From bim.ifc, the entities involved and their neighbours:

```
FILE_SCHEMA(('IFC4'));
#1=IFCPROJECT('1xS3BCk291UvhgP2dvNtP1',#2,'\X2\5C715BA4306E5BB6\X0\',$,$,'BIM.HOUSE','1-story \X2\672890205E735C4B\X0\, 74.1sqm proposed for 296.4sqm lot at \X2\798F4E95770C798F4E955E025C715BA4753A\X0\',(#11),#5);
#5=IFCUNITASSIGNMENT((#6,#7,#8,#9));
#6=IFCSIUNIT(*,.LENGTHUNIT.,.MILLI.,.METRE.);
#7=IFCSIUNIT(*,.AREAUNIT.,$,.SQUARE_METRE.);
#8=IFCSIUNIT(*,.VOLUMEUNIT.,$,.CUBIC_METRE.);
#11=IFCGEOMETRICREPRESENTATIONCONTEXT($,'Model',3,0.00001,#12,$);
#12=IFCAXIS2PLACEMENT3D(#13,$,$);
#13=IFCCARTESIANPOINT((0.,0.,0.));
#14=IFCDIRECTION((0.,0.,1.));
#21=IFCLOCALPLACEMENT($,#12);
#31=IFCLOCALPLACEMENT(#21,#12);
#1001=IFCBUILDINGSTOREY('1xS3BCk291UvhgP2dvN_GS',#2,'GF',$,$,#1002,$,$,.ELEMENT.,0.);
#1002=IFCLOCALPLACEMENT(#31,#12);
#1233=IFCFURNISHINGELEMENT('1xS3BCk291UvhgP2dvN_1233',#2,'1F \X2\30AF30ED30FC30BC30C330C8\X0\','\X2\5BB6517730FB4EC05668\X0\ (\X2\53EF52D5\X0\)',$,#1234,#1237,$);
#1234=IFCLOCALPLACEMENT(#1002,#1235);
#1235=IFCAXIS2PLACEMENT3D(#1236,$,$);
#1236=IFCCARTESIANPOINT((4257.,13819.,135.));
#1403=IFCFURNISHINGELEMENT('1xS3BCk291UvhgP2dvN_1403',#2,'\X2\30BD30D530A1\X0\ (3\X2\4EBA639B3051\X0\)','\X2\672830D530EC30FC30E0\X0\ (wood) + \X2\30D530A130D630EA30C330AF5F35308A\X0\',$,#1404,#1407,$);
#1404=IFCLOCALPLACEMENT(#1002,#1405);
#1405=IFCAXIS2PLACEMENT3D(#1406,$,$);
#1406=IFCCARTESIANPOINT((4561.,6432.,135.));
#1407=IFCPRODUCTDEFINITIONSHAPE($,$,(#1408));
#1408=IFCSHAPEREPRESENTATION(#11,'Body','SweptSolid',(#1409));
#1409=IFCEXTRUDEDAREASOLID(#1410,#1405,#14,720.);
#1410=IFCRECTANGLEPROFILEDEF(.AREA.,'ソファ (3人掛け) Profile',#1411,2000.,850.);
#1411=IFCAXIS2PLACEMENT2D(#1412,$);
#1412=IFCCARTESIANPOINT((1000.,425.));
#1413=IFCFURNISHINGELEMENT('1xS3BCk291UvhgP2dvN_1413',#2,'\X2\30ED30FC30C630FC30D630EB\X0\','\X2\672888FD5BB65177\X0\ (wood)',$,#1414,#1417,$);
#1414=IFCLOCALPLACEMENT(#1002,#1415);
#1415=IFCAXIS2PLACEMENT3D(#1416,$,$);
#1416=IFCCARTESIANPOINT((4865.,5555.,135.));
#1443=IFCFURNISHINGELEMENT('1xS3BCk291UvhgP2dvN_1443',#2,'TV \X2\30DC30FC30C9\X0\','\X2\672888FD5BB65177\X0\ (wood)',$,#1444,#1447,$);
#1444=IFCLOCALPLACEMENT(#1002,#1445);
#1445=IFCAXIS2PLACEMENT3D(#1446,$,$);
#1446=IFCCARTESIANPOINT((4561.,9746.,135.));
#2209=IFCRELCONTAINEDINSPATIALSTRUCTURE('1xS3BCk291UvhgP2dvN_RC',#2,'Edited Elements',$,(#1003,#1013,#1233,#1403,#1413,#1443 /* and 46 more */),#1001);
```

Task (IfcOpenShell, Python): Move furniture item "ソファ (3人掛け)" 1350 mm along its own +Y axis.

```python
import ifcopenshell
import ifcopenshell.api.geometry
import ifcopenshell.util.placement
import ifcopenshell.util.unit

model = ifcopenshell.open("bim.ifc")
unit_scale = ifcopenshell.util.unit.calculate_unit_scale(model)

item = model.by_guid("1xS3BCk291UvhgP2dvN_1403")
matrix = ifcopenshell.util.placement.get_local_placement(item.ObjectPlacement)
matrix[:3, 3] += matrix[:3, 1] * 1.35 / unit_scale
ifcopenshell.api.geometry.edit_object_placement(model, product=item, matrix=matrix, is_si=False)

print(ifcopenshell.util.placement.get_local_placement(item.ObjectPlacement).round(3) + 0.0)

model.write("bim_edited.ifc")
```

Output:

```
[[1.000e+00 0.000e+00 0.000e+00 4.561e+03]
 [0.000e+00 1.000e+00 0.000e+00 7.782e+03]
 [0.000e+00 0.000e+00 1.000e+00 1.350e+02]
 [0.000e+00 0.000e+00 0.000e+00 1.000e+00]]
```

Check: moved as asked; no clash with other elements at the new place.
